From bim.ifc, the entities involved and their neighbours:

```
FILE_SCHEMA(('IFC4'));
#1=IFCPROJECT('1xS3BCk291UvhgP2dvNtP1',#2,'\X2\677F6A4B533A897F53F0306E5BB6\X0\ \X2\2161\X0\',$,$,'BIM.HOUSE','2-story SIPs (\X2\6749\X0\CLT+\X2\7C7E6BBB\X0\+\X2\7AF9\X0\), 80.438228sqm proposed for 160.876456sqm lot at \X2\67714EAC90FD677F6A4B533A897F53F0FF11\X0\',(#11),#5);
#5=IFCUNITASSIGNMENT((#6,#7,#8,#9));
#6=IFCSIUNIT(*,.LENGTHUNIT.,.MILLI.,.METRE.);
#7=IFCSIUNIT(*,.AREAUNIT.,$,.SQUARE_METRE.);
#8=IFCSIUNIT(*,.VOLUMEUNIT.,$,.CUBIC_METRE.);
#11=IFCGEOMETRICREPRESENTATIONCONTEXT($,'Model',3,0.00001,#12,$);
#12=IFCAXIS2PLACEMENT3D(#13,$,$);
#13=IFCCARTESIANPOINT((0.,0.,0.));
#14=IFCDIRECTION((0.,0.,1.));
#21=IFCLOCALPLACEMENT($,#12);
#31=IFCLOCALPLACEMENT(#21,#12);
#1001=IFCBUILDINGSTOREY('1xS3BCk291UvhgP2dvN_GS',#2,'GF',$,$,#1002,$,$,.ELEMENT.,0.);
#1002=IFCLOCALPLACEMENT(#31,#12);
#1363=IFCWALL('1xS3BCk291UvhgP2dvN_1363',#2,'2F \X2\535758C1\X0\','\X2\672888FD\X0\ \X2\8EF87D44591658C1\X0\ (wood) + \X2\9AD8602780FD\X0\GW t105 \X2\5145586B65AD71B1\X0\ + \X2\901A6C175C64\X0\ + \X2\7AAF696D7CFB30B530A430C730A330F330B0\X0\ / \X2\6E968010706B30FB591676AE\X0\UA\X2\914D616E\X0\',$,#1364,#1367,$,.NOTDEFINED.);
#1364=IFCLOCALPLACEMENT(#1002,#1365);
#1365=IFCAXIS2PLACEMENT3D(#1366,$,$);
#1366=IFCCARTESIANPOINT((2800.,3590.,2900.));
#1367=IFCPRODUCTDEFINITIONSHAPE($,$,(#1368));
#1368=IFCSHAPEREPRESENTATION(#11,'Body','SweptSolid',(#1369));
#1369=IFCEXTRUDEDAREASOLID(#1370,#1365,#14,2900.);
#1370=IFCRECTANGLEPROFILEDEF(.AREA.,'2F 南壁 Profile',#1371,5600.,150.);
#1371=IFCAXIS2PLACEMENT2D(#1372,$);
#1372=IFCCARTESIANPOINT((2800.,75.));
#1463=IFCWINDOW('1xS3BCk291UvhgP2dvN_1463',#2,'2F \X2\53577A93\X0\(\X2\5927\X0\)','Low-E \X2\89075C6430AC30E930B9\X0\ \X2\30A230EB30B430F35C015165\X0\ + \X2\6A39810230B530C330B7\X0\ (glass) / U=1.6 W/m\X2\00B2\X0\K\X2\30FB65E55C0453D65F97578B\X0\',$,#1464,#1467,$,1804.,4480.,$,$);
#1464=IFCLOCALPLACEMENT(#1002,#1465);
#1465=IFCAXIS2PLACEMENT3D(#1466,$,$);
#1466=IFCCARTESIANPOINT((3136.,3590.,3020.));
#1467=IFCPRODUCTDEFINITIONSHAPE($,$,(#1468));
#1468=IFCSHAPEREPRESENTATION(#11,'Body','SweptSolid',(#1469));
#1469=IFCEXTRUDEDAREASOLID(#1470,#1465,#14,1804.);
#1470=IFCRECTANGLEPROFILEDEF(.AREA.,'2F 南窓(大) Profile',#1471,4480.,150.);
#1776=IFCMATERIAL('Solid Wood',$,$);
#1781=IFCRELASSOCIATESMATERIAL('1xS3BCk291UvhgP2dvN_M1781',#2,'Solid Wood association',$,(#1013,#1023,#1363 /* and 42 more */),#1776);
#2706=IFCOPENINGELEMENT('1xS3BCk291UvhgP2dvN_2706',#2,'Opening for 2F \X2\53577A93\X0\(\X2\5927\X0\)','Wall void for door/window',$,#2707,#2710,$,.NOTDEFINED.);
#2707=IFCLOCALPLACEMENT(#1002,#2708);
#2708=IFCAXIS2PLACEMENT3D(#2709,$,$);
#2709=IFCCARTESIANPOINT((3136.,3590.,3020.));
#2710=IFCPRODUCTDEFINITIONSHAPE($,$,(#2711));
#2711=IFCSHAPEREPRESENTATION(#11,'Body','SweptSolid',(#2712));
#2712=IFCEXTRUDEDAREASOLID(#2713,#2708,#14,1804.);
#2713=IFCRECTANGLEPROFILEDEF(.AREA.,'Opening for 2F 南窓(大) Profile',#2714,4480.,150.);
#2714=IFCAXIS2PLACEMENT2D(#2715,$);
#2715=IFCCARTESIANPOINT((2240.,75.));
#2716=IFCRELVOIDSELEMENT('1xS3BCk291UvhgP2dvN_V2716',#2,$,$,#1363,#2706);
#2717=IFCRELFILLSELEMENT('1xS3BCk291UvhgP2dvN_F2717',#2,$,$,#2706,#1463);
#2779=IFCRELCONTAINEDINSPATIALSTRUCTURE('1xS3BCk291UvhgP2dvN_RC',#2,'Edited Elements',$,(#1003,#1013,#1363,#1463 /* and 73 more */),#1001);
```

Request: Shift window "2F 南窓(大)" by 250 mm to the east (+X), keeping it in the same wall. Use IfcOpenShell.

```python
import ifcopenshell
import ifcopenshell.api.geometry
import ifcopenshell.util.placement
import ifcopenshell.util.unit

model = ifcopenshell.open("bim.ifc")
unit_scale = ifcopenshell.util.unit.calculate_unit_scale(model)

window = model.by_guid("1xS3BCk291UvhgP2dvN_1463")
opening = window.FillsVoids[0].RelatingOpeningElement
wall = opening.VoidsElements[0].RelatingBuildingElement

wall_matrix = ifcopenshell.util.placement.get_local_placement(wall.ObjectPlacement)
shift = wall_matrix[:3, 0] * 0.25 / unit_scale
before = ifcopenshell.util.placement.get_local_placement(window.ObjectPlacement)[:3, 3].copy()

# The window is not placed relative to its opening, so move both.
for product in (opening, window):
    matrix = ifcopenshell.util.placement.get_local_placement(product.ObjectPlacement)
    matrix[:3, 3] += shift
    ifcopenshell.api.geometry.edit_object_placement(model, product=product, matrix=matrix, is_si=False)

after = ifcopenshell.util.placement.get_local_placement(window.ObjectPlacement)[:3, 3]
print("window moved by", (after - before).round(3) + 0.0)

model.write("bim_v2.ifc")
```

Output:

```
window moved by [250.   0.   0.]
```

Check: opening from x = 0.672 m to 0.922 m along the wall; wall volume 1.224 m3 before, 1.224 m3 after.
